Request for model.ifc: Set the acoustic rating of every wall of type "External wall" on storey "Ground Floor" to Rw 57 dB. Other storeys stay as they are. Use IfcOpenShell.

First a look at what the model holds.

```python
import ifcopenshell
import ifcopenshell.util.element

model = ifcopenshell.open("model.ifc")
print(model.schema)
storey = next(s for s in model.by_type("IfcBuildingStorey") if s.Name == "Ground Floor")
walls = [e for e in ifcopenshell.util.element.get_decomposition(storey) if e.is_a("IfcWall")]
seen = {}
for e in walls:
    element_type = ifcopenshell.util.element.get_type(e)
    key = (element_type.Name if element_type != e and element_type else None, ifcopenshell.util.element.get_pset(e, "Pset_WallCommon", "AcousticRating"))
    seen[key] = seen.get(key, 0) + 1
for (name, value), count in sorted(seen.items(), key=str):
    print(count, "x", name, "|", value)
```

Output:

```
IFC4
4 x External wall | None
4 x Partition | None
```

```python
import ifcopenshell
import ifcopenshell.api.pset
import ifcopenshell.util.element

model = ifcopenshell.open("model.ifc")

storey = next(s for s in model.by_type("IfcBuildingStorey") if s.Name == "Ground Floor")
walls = [e for e in ifcopenshell.util.element.get_decomposition(storey) if e.is_a("IfcWall")]

count = 0
for e in walls:
    element_type = ifcopenshell.util.element.get_type(e)
    if element_type in (None, e) or element_type.Name != "External wall":
        continue
    # add_pset returns the element's existing set when there is one.
    pset = ifcopenshell.api.pset.add_pset(model, product=e, name="Pset_WallCommon")
    ifcopenshell.api.pset.edit_pset(model, pset=pset, properties={"AcousticRating": "Rw 57 dB"})
    count += 1

print(count, "walls updated")

model.write("model_rev.ifc")
```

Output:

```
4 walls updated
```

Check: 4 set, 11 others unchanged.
